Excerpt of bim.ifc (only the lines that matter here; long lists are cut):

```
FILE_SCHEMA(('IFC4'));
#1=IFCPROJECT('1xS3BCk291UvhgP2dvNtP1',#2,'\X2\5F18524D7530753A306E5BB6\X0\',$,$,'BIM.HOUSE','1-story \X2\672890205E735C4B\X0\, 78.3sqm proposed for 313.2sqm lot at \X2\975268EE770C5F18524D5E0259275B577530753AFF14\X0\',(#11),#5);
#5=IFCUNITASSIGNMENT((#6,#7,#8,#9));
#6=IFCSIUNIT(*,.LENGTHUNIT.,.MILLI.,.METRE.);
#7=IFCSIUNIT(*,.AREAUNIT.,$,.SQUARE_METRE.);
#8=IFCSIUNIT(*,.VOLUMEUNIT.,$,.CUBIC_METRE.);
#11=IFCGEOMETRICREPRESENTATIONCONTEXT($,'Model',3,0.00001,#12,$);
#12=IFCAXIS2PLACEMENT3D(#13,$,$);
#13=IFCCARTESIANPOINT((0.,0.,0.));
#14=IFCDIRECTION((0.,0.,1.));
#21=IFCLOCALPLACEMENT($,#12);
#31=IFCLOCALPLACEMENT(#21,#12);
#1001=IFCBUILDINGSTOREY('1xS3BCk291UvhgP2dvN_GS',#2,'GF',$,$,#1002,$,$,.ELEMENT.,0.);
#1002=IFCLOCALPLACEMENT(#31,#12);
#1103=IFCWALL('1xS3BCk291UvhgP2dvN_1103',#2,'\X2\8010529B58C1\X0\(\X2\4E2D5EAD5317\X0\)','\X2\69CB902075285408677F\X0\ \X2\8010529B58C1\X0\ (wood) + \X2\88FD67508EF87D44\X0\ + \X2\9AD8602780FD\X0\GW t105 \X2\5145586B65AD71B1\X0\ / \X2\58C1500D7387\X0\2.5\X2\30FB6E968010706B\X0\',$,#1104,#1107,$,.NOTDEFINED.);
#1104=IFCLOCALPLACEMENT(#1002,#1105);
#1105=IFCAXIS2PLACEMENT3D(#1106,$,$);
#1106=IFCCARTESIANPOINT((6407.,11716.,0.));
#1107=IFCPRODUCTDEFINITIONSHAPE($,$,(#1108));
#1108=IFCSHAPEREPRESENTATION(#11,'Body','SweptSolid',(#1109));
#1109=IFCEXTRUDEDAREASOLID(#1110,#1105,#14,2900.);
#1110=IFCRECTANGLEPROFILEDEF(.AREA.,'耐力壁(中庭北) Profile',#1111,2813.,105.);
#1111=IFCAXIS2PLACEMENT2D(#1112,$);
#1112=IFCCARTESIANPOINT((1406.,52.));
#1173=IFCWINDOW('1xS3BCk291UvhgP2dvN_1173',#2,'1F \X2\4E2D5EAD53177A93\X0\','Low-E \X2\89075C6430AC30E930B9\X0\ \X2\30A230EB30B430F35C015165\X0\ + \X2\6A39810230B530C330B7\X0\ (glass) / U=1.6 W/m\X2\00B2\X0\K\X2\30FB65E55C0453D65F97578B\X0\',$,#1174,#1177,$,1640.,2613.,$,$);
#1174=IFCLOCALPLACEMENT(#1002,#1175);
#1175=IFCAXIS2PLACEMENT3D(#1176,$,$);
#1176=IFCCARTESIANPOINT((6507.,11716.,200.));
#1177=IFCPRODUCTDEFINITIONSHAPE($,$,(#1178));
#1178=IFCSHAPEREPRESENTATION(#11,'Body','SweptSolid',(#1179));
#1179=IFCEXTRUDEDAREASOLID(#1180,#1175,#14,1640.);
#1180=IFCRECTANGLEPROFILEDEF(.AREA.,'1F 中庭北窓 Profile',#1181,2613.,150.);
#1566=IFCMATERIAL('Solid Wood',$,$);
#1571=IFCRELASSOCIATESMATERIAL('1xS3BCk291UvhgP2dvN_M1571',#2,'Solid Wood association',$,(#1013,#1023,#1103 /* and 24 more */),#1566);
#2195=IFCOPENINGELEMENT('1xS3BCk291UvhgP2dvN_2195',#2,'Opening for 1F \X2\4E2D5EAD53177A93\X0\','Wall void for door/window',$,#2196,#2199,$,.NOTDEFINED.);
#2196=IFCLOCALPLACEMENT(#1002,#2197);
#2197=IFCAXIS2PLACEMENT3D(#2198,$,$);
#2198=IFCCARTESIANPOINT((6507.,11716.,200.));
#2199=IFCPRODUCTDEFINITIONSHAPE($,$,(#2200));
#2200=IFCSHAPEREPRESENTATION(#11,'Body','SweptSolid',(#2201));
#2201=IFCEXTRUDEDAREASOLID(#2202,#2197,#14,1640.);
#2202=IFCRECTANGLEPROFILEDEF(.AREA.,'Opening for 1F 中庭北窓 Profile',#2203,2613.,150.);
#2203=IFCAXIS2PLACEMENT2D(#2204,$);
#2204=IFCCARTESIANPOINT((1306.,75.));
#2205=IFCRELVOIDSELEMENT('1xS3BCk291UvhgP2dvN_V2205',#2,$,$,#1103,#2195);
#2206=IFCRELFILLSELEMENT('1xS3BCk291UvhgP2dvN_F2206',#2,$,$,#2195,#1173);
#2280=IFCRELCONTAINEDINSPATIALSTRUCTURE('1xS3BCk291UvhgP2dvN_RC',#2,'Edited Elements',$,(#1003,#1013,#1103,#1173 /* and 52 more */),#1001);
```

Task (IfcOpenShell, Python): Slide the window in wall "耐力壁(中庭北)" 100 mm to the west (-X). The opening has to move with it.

```python
import ifcopenshell
import ifcopenshell.api.geometry
import ifcopenshell.util.placement
import ifcopenshell.util.unit

model = ifcopenshell.open("bim.ifc")
unit_scale = ifcopenshell.util.unit.calculate_unit_scale(model)

window = model.by_guid("1xS3BCk291UvhgP2dvN_1173")
opening = window.FillsVoids[0].RelatingOpeningElement
wall = opening.VoidsElements[0].RelatingBuildingElement

wall_matrix = ifcopenshell.util.placement.get_local_placement(wall.ObjectPlacement)
shift = wall_matrix[:3, 0] * -0.1 / unit_scale
before = ifcopenshell.util.placement.get_local_placement(window.ObjectPlacement)[:3, 3].copy()

# The window is not placed relative to its opening, so move both.
for product in (opening, window):
    matrix = ifcopenshell.util.placement.get_local_placement(product.ObjectPlacement)
    matrix[:3, 3] += shift
    ifcopenshell.api.geometry.edit_object_placement(model, product=product, matrix=matrix, is_si=False)

after = ifcopenshell.util.placement.get_local_placement(window.ObjectPlacement)[:3, 3]
print("window moved by", (after - before).round(3) + 0.0)

model.write("bim-out.ifc")
```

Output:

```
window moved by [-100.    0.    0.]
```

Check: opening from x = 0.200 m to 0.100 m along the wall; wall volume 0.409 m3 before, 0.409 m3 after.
